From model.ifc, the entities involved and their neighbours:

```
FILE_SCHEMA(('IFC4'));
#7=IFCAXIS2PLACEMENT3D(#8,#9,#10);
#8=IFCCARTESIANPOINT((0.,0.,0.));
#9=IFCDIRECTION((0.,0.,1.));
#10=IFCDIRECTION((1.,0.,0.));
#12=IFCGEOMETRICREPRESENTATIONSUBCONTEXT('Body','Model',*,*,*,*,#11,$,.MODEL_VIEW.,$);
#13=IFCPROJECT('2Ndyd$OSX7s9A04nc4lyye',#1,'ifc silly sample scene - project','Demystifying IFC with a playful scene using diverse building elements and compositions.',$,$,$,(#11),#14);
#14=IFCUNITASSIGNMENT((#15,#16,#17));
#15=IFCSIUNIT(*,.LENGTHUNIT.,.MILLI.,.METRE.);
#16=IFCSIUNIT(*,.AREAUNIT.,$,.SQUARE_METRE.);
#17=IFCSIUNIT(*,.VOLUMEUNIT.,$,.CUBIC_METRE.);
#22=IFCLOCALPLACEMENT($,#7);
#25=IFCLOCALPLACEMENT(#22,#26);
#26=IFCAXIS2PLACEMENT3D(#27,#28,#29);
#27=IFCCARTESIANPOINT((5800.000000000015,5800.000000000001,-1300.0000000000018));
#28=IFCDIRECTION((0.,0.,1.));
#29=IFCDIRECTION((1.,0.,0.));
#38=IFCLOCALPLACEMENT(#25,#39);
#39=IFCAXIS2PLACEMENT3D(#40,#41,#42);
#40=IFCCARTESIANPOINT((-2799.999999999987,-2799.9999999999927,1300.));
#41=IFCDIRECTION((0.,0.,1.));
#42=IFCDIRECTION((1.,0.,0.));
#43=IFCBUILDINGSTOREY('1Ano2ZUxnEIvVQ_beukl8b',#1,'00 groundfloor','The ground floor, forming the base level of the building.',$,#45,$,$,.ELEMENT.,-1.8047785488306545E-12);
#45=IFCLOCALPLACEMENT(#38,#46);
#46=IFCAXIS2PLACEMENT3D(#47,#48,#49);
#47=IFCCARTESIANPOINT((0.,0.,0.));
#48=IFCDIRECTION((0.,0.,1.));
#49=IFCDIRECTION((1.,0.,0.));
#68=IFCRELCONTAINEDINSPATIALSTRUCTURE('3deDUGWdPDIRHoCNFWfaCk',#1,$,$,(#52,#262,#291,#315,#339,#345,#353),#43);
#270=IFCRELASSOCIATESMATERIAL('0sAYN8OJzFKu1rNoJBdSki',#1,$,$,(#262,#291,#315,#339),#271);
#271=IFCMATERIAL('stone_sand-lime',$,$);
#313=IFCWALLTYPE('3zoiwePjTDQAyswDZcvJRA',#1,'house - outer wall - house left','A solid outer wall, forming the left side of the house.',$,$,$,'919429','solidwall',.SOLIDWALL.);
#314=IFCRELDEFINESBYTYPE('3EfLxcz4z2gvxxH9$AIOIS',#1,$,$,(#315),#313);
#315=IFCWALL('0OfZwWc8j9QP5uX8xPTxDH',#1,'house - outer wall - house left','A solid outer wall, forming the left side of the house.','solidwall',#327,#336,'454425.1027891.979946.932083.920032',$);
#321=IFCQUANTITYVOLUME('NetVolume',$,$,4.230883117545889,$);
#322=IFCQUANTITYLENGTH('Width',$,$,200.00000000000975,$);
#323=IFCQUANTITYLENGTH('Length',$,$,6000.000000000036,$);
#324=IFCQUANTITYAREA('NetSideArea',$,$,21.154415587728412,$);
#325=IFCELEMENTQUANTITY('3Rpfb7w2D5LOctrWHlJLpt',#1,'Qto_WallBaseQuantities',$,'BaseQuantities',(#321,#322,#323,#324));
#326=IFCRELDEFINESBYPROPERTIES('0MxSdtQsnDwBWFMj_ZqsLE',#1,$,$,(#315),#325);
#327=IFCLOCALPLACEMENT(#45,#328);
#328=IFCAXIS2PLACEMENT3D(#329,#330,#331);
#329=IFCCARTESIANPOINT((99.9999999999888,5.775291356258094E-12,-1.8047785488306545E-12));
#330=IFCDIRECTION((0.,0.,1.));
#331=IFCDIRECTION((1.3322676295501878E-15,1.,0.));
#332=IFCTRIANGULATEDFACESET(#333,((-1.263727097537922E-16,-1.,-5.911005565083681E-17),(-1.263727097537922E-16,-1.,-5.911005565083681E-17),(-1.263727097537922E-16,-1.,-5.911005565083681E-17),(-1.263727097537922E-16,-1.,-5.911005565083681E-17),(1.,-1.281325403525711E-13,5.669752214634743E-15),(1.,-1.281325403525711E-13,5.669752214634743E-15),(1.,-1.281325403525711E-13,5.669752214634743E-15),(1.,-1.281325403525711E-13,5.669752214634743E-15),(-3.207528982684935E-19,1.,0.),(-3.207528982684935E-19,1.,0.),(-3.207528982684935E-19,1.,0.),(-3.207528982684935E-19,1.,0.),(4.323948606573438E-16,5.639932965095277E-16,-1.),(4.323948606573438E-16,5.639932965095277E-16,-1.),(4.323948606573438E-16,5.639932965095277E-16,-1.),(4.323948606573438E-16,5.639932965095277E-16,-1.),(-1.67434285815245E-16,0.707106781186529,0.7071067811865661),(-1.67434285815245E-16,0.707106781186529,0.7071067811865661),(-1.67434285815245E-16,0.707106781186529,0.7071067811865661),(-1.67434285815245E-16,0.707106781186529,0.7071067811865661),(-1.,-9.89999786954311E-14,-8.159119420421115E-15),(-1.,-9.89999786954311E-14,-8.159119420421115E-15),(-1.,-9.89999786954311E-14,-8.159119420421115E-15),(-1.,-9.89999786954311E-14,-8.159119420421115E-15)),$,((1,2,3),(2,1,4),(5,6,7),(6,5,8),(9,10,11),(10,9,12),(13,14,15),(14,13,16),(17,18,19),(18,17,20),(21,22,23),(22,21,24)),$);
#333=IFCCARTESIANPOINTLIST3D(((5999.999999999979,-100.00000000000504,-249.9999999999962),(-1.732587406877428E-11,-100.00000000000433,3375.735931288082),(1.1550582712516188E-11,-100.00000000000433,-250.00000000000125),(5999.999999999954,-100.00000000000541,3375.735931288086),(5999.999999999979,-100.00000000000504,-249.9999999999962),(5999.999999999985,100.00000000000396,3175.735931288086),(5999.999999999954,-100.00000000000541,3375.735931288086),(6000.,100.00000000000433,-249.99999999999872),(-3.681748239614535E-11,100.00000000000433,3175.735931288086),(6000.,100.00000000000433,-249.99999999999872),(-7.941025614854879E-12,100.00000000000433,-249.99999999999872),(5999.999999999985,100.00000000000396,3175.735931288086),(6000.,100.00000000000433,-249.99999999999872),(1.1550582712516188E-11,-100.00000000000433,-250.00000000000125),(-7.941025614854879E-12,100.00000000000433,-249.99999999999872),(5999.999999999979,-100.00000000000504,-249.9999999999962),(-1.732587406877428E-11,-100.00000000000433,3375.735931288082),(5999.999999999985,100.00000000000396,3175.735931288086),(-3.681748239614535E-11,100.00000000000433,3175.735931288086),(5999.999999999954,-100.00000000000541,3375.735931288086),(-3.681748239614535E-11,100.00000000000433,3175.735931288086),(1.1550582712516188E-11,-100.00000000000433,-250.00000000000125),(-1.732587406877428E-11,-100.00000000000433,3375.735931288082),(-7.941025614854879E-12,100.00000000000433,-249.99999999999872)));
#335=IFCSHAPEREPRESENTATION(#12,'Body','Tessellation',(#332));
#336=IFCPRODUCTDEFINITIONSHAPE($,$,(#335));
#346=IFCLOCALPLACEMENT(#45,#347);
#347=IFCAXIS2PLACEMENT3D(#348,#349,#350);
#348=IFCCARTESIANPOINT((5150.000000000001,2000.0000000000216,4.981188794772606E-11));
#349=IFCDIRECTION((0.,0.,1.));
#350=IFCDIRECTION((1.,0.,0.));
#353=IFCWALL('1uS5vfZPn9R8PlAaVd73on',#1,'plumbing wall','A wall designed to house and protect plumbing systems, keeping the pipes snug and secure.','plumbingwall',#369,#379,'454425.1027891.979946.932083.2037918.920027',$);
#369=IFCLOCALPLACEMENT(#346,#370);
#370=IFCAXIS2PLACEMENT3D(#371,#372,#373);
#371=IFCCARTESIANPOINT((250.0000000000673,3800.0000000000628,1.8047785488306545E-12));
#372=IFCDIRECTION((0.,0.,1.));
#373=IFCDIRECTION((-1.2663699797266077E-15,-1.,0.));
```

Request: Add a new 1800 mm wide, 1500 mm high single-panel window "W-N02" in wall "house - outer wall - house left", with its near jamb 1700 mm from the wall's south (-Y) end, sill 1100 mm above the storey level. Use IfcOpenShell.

```python
import numpy as np
import ifcopenshell
import ifcopenshell.api.feature
import ifcopenshell.api.geometry
import ifcopenshell.api.pset
import ifcopenshell.api.root
import ifcopenshell.api.spatial
import ifcopenshell.geom
import ifcopenshell.util.element
import ifcopenshell.util.placement
import ifcopenshell.util.representation
import ifcopenshell.util.shape
import ifcopenshell.util.unit

model = ifcopenshell.open("model.ifc")
unit_scale = ifcopenshell.util.unit.calculate_unit_scale(model)
area_scale = ifcopenshell.util.unit.calculate_unit_scale(model, "AREAUNIT")
volume_scale = ifcopenshell.util.unit.calculate_unit_scale(model, "VOLUMEUNIT")
settings = ifcopenshell.geom.settings()


def volume(element):
    """Net volume in cubic metres, openings subtracted."""
    shape = ifcopenshell.geom.create_shape(settings, element)
    return ifcopenshell.util.shape.get_volume(shape.geometry)


wall = model.by_guid("0OfZwWc8j9QP5uX8xPTxDH")
storey = ifcopenshell.util.element.get_container(wall, ifc_class="IfcBuildingStorey")
context = ifcopenshell.util.representation.get_context(model, "Model", "Body", "MODEL_VIEW")
before = volume(wall)

width, height, from_end, sill = 1.8, 1.5, 1.7, 1.1  # metres

# The wall runs along its own X axis, and the end named is its -X end.
wall_shape = ifcopenshell.geom.create_shape(settings, wall)
x, y, z = ifcopenshell.util.shape.get_vertices(wall_shape.geometry).T
start = x.min() + from_end
face, thickness = float(y.min()), float(y.max() - y.min())
wall_matrix = ifcopenshell.util.placement.get_local_placement(wall.ObjectPlacement)
level = ifcopenshell.util.placement.get_local_placement(storey.ObjectPlacement)[2, 3]


def in_wall(x, y):
    """Placement at x, y metres in the wall's axes, at sill height."""
    matrix = wall_matrix.copy()
    matrix[:, 3] = wall_matrix @ np.array([x / unit_scale, y / unit_scale, 0.0, 1.0])
    matrix[2, 3] = level + sill / unit_scale
    return matrix


# Opening: a box that overshoots both wall faces by 50 mm.
opening = ifcopenshell.api.root.create_entity(model, ifc_class="IfcOpeningElement", predefined_type="OPENING")
box = ifcopenshell.api.geometry.add_wall_representation(
    model, context=context, length=width, height=height, thickness=thickness + 0.1
)
ifcopenshell.api.geometry.assign_representation(model, product=opening, representation=box)
ifcopenshell.api.geometry.edit_object_placement(model, product=opening, matrix=in_wall(start, face - 0.05), is_si=False)
ifcopenshell.api.feature.add_feature(model, feature=opening, element=wall)

window = ifcopenshell.api.root.create_entity(model, ifc_class="IfcWindow", name="W-N02", predefined_type="WINDOW")
window.OverallWidth, window.OverallHeight = width / unit_scale, height / unit_scale
window.PartitioningType = "SINGLE_PANEL"
body = ifcopenshell.api.geometry.add_window_representation(
    model,
    context=context,
    overall_width=window.OverallWidth,
    overall_height=window.OverallHeight,
    partition_type="SINGLE_PANEL",
)
ifcopenshell.api.geometry.assign_representation(model, product=window, representation=body)
ifcopenshell.api.spatial.assign_container(model, products=[window], relating_structure=storey)
ifcopenshell.api.feature.add_filling(model, opening=opening, element=window)

# Centre the window in the wall's thickness.
ifcopenshell.api.geometry.edit_object_placement(model, product=window, matrix=in_wall(start, face), is_si=False)
window_shape = ifcopenshell.geom.create_shape(settings, window)
depth = ifcopenshell.util.shape.get_vertices(window_shape.geometry)[:, 1]
offset = face + thickness / 2 - (depth.min() + depth.max()) / 2
ifcopenshell.api.geometry.edit_object_placement(model, product=window, matrix=in_wall(start, offset), is_si=False)

after = volume(wall)

# Update the wall's stored quantities.
qto = model.by_id(ifcopenshell.util.element.get_pset(wall, "Qto_WallBaseQuantities", should_inherit=False)["id"])
ifcopenshell.api.pset.edit_qto(model, qto=qto, properties={
    "NetVolume": after / volume_scale,
    "NetSideArea": after / thickness / area_scale,
})

print(f"wall volume {before:.3f} -> {after:.3f} m3")

model.write("model_updated.ifc")
```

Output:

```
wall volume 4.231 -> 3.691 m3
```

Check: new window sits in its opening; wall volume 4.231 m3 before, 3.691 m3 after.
